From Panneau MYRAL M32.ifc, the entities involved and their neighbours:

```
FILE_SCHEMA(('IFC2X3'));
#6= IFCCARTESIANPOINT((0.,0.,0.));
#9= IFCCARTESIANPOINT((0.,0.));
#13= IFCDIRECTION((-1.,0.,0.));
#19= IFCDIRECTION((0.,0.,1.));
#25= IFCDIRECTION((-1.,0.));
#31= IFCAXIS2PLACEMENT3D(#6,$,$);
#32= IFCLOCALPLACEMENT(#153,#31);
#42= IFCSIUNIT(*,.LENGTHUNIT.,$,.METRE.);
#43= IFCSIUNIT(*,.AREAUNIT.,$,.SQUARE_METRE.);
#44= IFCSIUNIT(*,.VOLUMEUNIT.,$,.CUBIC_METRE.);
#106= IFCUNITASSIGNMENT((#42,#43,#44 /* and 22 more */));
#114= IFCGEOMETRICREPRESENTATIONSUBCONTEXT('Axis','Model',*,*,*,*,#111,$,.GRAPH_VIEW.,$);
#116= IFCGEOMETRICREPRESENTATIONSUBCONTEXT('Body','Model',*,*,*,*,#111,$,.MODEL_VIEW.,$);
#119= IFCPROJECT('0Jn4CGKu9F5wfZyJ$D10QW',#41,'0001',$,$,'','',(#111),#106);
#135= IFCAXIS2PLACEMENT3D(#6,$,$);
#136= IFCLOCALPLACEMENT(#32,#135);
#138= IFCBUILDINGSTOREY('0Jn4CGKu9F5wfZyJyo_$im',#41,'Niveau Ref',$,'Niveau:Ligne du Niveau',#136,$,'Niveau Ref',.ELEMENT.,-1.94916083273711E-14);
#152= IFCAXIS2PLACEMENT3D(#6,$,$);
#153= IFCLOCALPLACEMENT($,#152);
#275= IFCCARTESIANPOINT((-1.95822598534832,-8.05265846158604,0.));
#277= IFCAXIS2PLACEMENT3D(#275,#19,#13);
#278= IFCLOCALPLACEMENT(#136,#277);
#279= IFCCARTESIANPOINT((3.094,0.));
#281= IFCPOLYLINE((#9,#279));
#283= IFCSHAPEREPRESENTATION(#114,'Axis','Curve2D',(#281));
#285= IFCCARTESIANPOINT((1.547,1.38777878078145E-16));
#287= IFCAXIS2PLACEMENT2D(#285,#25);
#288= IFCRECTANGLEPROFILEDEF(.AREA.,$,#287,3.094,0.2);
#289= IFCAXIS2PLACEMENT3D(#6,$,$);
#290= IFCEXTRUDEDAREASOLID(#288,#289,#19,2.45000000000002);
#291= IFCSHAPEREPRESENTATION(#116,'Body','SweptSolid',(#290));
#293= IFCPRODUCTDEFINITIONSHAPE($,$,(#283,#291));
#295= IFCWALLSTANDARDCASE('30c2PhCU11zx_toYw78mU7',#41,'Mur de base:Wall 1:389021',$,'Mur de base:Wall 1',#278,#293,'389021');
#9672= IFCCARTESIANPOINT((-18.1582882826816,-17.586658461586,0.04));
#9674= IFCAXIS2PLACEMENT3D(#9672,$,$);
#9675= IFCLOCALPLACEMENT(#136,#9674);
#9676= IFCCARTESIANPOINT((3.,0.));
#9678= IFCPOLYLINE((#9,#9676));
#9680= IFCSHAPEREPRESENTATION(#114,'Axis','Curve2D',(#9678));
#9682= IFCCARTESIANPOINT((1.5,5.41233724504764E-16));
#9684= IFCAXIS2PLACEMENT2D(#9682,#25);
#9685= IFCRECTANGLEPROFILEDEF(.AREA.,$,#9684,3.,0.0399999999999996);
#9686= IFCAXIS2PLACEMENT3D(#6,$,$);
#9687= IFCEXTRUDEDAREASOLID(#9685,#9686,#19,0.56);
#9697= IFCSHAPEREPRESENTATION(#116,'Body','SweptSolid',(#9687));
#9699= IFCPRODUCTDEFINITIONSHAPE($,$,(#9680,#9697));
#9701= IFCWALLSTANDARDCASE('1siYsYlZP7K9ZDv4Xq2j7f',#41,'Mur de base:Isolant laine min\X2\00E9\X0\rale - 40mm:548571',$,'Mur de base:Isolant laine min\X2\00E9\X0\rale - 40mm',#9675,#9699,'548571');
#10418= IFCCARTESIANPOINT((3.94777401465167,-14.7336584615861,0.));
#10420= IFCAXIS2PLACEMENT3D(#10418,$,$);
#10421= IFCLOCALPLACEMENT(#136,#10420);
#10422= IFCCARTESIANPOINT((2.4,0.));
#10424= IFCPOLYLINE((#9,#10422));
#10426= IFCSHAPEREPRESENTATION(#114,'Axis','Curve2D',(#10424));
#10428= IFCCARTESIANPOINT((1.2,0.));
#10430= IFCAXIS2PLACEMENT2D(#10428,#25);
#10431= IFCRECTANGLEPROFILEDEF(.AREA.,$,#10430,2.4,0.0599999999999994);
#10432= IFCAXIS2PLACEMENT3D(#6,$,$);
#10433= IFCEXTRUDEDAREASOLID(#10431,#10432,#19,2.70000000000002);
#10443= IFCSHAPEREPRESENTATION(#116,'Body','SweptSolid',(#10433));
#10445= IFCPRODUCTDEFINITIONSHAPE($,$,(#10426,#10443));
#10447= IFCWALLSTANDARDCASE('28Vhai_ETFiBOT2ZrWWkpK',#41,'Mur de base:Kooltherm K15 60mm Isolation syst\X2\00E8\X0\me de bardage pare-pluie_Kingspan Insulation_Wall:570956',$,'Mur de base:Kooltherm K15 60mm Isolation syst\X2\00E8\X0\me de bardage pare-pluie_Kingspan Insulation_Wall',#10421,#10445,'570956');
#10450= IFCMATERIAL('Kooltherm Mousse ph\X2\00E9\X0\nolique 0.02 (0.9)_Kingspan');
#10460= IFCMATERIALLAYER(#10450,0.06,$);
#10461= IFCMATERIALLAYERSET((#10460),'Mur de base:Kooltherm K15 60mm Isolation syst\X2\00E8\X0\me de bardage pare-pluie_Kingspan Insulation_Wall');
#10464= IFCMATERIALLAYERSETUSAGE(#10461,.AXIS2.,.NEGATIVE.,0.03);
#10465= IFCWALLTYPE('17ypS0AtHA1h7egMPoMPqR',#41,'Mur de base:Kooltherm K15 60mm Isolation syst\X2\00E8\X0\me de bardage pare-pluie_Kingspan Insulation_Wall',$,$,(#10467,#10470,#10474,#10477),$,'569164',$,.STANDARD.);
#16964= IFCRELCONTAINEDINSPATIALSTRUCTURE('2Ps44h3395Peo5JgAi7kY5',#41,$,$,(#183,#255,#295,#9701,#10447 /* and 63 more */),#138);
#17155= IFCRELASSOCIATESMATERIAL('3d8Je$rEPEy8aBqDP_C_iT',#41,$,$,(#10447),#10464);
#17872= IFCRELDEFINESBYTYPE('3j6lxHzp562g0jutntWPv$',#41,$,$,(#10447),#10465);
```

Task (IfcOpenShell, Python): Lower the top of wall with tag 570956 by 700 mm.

```python
import ifcopenshell
import ifcopenshell.geom
import ifcopenshell.util.representation
import ifcopenshell.util.shape

model = ifcopenshell.open("Panneau MYRAL M32.ifc")
settings = ifcopenshell.geom.settings()


def volume(element):
    """Net volume in cubic metres, openings subtracted."""
    shape = ifcopenshell.geom.create_shape(settings, element)
    return ifcopenshell.util.shape.get_volume(shape.geometry)


wall = model.by_id(10447)
before = volume(wall)

body = ifcopenshell.util.representation.get_representation(wall, "Model", "Body")
solid = body.Items[0]
old_height = solid.Depth
solid.Depth -= 0.7
after = volume(wall)

print(f"height {old_height:g} -> {solid.Depth:g}, volume {before:.3f} -> {after:.3f} m3")

model.write("Panneau MYRAL M32_updated.ifc")
```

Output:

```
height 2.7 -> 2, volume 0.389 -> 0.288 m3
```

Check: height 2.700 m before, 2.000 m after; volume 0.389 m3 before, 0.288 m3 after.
